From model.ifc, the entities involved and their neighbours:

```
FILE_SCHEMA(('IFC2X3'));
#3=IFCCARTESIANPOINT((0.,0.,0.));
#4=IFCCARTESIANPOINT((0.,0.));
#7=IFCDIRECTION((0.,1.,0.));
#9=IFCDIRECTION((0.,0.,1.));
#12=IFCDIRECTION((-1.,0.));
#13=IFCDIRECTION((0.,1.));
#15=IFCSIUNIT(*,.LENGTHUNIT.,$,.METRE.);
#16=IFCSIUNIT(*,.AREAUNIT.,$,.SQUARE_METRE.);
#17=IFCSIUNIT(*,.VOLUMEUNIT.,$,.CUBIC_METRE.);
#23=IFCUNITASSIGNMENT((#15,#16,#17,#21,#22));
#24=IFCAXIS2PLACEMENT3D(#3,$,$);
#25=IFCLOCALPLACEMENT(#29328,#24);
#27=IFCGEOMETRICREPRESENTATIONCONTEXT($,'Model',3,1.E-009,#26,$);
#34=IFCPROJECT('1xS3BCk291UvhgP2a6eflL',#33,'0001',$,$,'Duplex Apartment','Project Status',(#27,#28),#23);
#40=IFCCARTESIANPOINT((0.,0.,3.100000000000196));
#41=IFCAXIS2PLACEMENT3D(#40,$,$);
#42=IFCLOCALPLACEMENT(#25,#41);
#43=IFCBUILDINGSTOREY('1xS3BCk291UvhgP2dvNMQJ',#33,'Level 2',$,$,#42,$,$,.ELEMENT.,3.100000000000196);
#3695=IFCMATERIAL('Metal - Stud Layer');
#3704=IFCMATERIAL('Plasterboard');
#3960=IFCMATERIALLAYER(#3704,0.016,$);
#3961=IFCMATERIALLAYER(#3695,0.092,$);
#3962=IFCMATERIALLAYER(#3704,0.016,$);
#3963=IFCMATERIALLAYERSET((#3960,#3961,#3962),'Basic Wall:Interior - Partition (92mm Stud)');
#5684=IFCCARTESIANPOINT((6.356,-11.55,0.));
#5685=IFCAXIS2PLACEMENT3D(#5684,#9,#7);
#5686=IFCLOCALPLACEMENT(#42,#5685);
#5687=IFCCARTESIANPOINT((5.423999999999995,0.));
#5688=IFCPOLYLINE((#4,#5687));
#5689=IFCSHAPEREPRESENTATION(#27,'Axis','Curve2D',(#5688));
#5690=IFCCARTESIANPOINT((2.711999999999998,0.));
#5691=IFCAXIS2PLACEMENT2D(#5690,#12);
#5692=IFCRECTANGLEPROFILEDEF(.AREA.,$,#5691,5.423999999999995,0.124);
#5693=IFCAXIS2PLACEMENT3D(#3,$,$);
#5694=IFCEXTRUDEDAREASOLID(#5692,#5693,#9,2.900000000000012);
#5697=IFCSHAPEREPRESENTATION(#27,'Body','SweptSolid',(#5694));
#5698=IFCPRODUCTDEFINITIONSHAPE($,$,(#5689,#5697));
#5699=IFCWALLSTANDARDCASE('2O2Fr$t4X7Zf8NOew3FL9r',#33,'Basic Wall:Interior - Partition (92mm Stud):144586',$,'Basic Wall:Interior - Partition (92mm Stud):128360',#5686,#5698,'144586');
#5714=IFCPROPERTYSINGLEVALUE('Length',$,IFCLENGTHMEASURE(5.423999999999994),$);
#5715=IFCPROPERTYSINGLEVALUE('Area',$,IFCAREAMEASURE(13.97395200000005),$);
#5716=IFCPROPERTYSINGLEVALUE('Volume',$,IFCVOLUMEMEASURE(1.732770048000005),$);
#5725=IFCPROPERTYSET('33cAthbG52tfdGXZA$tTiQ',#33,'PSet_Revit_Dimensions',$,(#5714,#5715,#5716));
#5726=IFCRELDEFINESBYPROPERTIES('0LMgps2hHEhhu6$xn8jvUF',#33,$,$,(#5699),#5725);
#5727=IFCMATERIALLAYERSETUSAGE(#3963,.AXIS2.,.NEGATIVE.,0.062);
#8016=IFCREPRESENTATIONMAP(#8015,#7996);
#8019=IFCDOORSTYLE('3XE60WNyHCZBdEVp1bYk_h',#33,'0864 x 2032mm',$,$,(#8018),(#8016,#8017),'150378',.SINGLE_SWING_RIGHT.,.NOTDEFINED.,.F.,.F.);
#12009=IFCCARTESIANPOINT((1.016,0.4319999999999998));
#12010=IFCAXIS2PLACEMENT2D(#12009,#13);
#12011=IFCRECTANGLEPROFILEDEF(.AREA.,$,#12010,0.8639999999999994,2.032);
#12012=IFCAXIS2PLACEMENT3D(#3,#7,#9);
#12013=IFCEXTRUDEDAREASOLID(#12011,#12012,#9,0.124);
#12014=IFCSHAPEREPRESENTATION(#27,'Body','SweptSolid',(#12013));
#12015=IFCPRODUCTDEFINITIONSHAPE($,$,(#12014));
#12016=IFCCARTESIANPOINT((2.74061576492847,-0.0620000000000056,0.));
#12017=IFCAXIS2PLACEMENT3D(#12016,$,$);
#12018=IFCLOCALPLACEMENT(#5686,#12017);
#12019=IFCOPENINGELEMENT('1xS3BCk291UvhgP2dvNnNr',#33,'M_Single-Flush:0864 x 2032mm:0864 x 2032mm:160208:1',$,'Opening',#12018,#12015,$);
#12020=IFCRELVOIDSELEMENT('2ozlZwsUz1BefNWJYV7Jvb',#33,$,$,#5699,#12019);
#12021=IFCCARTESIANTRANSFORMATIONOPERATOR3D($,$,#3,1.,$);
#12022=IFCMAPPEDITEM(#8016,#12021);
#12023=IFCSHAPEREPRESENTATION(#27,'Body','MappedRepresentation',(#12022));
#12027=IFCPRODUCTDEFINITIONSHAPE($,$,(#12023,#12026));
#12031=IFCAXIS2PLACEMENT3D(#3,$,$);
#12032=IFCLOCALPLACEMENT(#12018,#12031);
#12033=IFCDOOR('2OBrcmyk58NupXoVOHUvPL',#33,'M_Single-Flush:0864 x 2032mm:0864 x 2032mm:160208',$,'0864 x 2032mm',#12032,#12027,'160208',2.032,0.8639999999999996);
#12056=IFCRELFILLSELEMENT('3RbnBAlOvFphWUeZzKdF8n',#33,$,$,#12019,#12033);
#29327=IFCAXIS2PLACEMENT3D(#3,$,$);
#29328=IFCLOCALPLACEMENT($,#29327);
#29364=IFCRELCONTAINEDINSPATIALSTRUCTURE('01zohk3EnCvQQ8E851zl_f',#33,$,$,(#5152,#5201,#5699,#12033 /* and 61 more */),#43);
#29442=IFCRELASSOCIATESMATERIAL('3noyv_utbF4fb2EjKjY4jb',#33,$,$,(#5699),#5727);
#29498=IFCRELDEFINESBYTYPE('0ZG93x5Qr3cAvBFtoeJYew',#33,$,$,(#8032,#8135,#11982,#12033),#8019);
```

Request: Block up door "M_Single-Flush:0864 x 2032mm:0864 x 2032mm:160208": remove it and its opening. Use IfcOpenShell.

```python
import ifcopenshell
import ifcopenshell.api.feature
import ifcopenshell.api.pset
import ifcopenshell.api.root
import ifcopenshell.geom
import ifcopenshell.util.element
import ifcopenshell.util.shape
import ifcopenshell.util.unit

model = ifcopenshell.open("model.ifc")
area_scale = ifcopenshell.util.unit.calculate_unit_scale(model, "AREAUNIT")
volume_scale = ifcopenshell.util.unit.calculate_unit_scale(model, "VOLUMEUNIT")
settings = ifcopenshell.geom.settings()


def volume(element):
    """Net volume in cubic metres, openings subtracted."""
    shape = ifcopenshell.geom.create_shape(settings, element)
    return ifcopenshell.util.shape.get_volume(shape.geometry)


door = model.by_guid("2OBrcmyk58NupXoVOHUvPL")
opening = door.FillsVoids[0].RelatingOpeningElement
wall = opening.VoidsElements[0].RelatingBuildingElement
before = volume(wall)

ifcopenshell.api.root.remove_product(model, product=door)
ifcopenshell.api.feature.remove_feature(model, feature=opening)

after = volume(wall)
thickness = 0.124  # wall thickness in metres

# Update the wall's stored quantities.
pset = model.by_id(ifcopenshell.util.element.get_pset(wall, "PSet_Revit_Dimensions", should_inherit=False)["id"])
ifcopenshell.api.pset.edit_pset(model, pset=pset, properties={
    "Area": model.create_entity("IfcAreaMeasure", after / thickness / area_scale),
    "Volume": model.create_entity("IfcVolumeMeasure", after / volume_scale),
})

print(f"wall volume {before:.3f} -> {after:.3f} m3")

model.write("model_v2.ifc")
```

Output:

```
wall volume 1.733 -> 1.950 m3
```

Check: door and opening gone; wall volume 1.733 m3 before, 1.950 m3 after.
